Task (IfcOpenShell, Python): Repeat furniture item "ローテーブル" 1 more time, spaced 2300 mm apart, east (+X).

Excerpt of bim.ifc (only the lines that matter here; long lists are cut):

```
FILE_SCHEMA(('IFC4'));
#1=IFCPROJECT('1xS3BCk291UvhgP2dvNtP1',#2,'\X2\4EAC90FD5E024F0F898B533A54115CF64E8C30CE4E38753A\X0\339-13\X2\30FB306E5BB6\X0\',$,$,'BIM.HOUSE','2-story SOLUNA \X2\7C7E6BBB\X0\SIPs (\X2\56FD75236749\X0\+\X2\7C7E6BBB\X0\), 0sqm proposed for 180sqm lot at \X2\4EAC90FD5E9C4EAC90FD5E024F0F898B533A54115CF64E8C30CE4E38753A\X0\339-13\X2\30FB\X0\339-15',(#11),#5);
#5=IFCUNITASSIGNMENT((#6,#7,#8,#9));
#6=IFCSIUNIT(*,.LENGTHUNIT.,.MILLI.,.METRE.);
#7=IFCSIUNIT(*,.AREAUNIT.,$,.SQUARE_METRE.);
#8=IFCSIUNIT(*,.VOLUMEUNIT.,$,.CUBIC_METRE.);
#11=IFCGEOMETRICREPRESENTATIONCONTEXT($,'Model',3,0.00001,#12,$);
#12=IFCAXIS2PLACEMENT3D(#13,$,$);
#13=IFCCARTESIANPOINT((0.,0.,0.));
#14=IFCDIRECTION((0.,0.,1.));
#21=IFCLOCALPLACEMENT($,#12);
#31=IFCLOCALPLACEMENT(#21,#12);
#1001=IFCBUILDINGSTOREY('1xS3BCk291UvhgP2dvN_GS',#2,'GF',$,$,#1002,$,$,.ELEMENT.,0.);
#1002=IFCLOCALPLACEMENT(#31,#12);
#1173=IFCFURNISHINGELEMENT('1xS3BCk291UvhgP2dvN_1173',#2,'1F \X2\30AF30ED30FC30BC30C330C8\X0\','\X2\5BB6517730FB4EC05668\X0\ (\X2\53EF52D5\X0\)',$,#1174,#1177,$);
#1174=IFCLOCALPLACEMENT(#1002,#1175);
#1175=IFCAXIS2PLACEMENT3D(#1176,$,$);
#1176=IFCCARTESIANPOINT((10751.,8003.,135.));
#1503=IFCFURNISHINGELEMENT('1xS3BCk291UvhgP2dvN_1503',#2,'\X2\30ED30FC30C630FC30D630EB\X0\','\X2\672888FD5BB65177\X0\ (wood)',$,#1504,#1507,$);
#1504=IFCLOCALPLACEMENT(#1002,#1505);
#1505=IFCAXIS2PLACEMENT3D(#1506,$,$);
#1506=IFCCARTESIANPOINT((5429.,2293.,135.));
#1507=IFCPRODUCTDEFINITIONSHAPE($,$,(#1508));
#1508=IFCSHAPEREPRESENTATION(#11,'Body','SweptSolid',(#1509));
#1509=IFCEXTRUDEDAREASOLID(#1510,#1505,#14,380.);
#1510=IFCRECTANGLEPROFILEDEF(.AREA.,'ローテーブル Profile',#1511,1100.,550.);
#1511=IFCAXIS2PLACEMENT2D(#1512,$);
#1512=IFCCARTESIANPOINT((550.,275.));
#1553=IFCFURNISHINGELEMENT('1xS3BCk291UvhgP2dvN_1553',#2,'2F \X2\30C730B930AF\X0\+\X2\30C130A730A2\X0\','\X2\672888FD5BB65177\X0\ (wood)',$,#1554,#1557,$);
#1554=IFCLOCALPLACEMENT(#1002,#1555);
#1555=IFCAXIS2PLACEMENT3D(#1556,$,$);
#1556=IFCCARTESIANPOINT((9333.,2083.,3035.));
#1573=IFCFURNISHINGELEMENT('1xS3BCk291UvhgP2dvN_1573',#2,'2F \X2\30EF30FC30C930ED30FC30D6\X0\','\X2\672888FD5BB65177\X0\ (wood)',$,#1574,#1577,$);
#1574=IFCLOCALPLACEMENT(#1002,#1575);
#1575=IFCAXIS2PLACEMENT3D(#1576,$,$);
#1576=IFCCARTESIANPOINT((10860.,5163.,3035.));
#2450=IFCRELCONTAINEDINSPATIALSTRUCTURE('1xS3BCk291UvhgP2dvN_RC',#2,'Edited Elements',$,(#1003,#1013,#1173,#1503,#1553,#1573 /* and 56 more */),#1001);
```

```python
import numpy as np
import ifcopenshell
import ifcopenshell.api.geometry
import ifcopenshell.api.root
import ifcopenshell.util.element
import ifcopenshell.util.placement

model = ifcopenshell.open("bim.ifc")


def reuse_history(source, copy):
    """copy_class also copies each property set's owner history, people and application; keep the originals."""
    for rel in copy.IsDefinedBy:
        if rel.is_a("IfcRelDefinesByProperties") and (history := rel.RelatingPropertyDefinition.OwnerHistory):
            rel.RelatingPropertyDefinition.OwnerHistory = source.OwnerHistory
            ifcopenshell.util.element.remove_deep2(model, history)


source = model.by_guid("1xS3BCk291UvhgP2dvN_1503")
base = ifcopenshell.util.placement.get_local_placement(source.ObjectPlacement)
step = np.array([1.0, 0.0, 0.0]) * 2300.0

for i in range(1, 2):
    copy = ifcopenshell.api.root.copy_class(model, product=source)
    copy.Representation = ifcopenshell.util.element.copy_deep(
        model, source.Representation, exclude=["IfcGeometricRepresentationContext", "IfcRepresentationMap"]
    )
    reuse_history(source, copy)
    matrix = base.copy()
    matrix[:3, 3] += i * step
    print("added at", matrix[:3, 3].round(3) + 0.0)
    ifcopenshell.api.geometry.edit_object_placement(model, product=copy, matrix=matrix, is_si=False)

model.write("bim_edited.ifc")
```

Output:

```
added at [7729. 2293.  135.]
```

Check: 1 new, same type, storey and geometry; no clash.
